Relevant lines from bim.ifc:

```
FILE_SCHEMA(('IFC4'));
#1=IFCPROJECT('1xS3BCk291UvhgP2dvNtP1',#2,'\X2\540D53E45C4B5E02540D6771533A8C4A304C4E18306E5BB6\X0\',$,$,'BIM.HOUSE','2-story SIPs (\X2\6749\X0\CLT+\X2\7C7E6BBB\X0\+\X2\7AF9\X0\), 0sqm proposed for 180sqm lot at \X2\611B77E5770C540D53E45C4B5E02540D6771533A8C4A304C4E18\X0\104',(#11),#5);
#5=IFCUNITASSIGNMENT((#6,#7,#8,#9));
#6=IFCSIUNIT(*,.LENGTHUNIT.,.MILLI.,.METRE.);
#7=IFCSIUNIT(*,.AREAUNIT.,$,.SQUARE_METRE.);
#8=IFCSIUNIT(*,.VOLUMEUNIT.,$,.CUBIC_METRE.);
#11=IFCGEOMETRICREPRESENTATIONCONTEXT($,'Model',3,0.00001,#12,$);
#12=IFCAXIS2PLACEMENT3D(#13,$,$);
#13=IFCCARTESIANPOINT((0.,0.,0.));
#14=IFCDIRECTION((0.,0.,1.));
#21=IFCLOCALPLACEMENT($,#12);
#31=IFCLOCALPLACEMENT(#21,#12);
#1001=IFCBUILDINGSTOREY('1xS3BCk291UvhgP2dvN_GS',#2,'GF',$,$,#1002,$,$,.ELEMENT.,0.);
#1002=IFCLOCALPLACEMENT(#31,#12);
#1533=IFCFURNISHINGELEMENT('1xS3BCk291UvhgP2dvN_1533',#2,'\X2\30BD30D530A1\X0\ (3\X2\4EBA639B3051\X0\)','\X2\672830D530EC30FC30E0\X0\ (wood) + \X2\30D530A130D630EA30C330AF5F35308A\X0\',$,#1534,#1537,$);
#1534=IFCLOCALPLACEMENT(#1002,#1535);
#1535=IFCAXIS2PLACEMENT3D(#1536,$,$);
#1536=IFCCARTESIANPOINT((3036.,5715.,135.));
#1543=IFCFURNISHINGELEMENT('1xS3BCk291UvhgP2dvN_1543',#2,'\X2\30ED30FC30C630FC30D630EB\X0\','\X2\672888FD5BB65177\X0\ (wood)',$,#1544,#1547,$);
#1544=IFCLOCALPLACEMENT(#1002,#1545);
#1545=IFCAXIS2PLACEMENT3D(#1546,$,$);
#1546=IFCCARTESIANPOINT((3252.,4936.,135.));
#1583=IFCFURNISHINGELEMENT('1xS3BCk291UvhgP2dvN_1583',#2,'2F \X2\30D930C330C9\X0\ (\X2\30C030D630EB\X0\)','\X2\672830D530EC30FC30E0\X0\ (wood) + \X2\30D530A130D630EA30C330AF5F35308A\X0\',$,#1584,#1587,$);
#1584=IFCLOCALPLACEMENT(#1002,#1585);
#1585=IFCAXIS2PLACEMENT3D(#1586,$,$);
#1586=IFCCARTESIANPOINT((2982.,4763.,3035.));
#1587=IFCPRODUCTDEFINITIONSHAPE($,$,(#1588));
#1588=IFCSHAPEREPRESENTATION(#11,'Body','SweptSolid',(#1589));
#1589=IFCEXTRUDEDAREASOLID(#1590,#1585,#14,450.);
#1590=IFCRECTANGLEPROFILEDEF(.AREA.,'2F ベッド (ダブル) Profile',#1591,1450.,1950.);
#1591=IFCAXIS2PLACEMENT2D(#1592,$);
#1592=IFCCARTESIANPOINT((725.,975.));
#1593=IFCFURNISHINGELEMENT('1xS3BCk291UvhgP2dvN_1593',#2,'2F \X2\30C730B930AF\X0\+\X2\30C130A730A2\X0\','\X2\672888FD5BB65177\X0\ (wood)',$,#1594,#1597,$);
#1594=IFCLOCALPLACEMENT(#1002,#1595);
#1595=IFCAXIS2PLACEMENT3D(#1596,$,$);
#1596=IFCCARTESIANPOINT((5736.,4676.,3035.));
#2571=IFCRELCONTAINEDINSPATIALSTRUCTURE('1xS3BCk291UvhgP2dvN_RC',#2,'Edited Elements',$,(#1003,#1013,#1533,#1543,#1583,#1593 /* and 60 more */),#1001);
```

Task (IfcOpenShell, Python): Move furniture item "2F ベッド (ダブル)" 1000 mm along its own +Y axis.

```python
import ifcopenshell
import ifcopenshell.api.geometry
import ifcopenshell.util.placement
import ifcopenshell.util.unit

model = ifcopenshell.open("bim.ifc")
unit_scale = ifcopenshell.util.unit.calculate_unit_scale(model)

item = model.by_guid("1xS3BCk291UvhgP2dvN_1583")
matrix = ifcopenshell.util.placement.get_local_placement(item.ObjectPlacement)
matrix[:3, 3] += matrix[:3, 1] * 1 / unit_scale
ifcopenshell.api.geometry.edit_object_placement(model, product=item, matrix=matrix, is_si=False)

print(ifcopenshell.util.placement.get_local_placement(item.ObjectPlacement).round(3) + 0.0)

model.write("bim-out.ifc")
```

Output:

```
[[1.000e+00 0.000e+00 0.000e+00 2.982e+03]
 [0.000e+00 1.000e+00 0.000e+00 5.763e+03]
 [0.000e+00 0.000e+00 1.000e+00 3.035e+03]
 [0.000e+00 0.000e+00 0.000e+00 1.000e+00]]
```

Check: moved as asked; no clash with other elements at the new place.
